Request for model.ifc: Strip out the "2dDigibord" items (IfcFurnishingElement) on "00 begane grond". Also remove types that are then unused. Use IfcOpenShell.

First a look at what the model holds.

```python
import ifcopenshell
import ifcopenshell.util.element

model = ifcopenshell.open("model.ifc")
print(model.schema)
storey = next(s for s in model.by_type("IfcBuildingStorey") if s.Name == "00 begane grond")
furniture = [e for e in ifcopenshell.util.element.get_decomposition(storey) if e.is_a("IfcFurnishingElement")]
seen = {}
for e in furniture:
    element_type = ifcopenshell.util.element.get_type(e)
    name = element_type.Name if element_type not in (None, e) else None
    seen[name] = seen.get(name, 0) + 1
for name, count in sorted(seen.items(), key=str):
    print(count, "x", name)
```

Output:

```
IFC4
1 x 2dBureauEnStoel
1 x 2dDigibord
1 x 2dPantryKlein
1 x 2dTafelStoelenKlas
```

```python
import ifcopenshell
import ifcopenshell.api.root
import ifcopenshell.util.element

model = ifcopenshell.open("model.ifc")

storey = next(s for s in model.by_type("IfcBuildingStorey") if s.Name == "00 begane grond")
furniture = [e for e in ifcopenshell.util.element.get_decomposition(storey) if e.is_a("IfcFurnishingElement")]
targets = [e for e in furniture if (t := ifcopenshell.util.element.get_type(e)) not in (None, e) and t.Name == "2dDigibord"]
types = {ifcopenshell.util.element.get_type(e) for e in targets} - {None, *targets}

for e in targets:
    ifcopenshell.api.root.remove_product(model, product=e)
print(len(targets), "removed")

unused = [t for t in types if not ifcopenshell.util.element.get_types(t)]
for t in unused:
    ifcopenshell.api.root.remove_product(model, product=t)
print(len(unused), "unused types removed")

model.write("model_edited.ifc")
```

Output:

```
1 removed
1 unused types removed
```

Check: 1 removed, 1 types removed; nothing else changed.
